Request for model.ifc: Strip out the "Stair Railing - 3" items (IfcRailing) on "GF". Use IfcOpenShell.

First a look at what the model holds.

```python
import ifcopenshell
import ifcopenshell.util.element

model = ifcopenshell.open("model.ifc")
print(model.schema)
storey = next(s for s in model.by_type("IfcBuildingStorey") if s.Name == "GF")
railings = [e for e in ifcopenshell.util.element.get_decomposition(storey) if e.is_a("IfcRailing")]
seen = {}
for e in railings:
    element_type = ifcopenshell.util.element.get_type(e)
    name = element_type.Name if element_type not in (None, e) else None
    seen[name] = seen.get(name, 0) + 1
for name, count in sorted(seen.items(), key=str):
    print(count, "x", name)
```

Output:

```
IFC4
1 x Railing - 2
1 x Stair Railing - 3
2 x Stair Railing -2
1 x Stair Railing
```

```python
import ifcopenshell
import ifcopenshell.api.root
import ifcopenshell.util.element

model = ifcopenshell.open("model.ifc")

storey = next(s for s in model.by_type("IfcBuildingStorey") if s.Name == "GF")
railings = [e for e in ifcopenshell.util.element.get_decomposition(storey) if e.is_a("IfcRailing")]
targets = [e for e in railings if (t := ifcopenshell.util.element.get_type(e)) not in (None, e) and t.Name == "Stair Railing - 3"]

for e in targets:
    ifcopenshell.api.root.remove_product(model, product=e)
print(len(targets), "removed")

model.write("model_rev.ifc")
```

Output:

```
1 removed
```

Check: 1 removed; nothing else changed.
